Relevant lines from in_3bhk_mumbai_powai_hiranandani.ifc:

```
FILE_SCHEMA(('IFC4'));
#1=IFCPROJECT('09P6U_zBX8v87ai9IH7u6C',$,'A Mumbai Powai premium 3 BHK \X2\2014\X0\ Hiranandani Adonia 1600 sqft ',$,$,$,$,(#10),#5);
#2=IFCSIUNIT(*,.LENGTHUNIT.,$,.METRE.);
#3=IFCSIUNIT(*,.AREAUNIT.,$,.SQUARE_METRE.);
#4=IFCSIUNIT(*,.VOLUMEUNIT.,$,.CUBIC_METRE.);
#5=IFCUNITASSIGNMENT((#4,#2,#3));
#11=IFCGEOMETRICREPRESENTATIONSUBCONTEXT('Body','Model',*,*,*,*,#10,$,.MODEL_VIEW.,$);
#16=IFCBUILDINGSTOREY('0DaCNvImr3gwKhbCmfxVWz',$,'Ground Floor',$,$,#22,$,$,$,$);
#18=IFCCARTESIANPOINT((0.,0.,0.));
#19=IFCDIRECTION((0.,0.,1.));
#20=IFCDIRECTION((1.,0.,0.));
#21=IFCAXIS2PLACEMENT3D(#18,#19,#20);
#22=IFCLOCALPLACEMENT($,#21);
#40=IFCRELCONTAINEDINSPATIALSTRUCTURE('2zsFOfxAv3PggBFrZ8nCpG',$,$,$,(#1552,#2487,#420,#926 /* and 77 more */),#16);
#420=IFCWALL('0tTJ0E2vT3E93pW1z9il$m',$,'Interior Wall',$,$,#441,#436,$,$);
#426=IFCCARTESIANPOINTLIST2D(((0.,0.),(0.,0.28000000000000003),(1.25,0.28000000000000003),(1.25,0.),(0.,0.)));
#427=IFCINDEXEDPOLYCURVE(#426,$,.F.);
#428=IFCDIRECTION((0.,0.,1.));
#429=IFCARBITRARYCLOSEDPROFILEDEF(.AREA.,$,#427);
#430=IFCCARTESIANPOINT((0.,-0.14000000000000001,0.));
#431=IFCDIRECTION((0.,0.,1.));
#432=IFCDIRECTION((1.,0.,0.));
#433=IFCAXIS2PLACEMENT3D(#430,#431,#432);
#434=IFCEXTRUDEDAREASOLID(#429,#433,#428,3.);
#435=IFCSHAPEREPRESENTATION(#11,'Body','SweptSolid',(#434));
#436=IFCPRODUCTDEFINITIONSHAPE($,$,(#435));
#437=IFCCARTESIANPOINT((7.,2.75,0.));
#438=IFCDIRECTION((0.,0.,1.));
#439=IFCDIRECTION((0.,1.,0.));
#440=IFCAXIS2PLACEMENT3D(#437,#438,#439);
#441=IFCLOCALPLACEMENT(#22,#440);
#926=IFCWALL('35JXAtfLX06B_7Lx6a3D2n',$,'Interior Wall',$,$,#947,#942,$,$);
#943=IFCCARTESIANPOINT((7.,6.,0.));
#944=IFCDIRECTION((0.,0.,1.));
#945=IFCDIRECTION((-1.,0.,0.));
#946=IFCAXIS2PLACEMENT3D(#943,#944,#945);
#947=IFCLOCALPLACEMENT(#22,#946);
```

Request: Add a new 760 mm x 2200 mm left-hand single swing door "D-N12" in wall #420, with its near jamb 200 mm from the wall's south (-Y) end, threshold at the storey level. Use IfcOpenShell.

```python
import numpy as np
import ifcopenshell
import ifcopenshell.api.feature
import ifcopenshell.api.geometry
import ifcopenshell.api.root
import ifcopenshell.api.spatial
import ifcopenshell.geom
import ifcopenshell.util.element
import ifcopenshell.util.placement
import ifcopenshell.util.representation
import ifcopenshell.util.shape
import ifcopenshell.util.unit

model = ifcopenshell.open("in_3bhk_mumbai_powai_hiranandani.ifc")
unit_scale = ifcopenshell.util.unit.calculate_unit_scale(model)
settings = ifcopenshell.geom.settings()


def volume(element):
    """Net volume in cubic metres, openings subtracted."""
    shape = ifcopenshell.geom.create_shape(settings, element)
    return ifcopenshell.util.shape.get_volume(shape.geometry)


wall = model.by_id(420)
storey = ifcopenshell.util.element.get_container(wall, ifc_class="IfcBuildingStorey")
context = ifcopenshell.util.representation.get_context(model, "Model", "Body", "MODEL_VIEW")
before = volume(wall)

width, height, from_end, sill = 0.76, 2.2, 0.2, 0.0  # metres

# The wall runs along its own X axis, and the end named is its -X end.
wall_shape = ifcopenshell.geom.create_shape(settings, wall)
x, y, z = ifcopenshell.util.shape.get_vertices(wall_shape.geometry).T
start = x.min() + from_end
face, thickness = float(y.min()), float(y.max() - y.min())
wall_matrix = ifcopenshell.util.placement.get_local_placement(wall.ObjectPlacement)
level = ifcopenshell.util.placement.get_local_placement(storey.ObjectPlacement)[2, 3]


def in_wall(x, y):
    """Placement at x, y metres in the wall's axes, at sill height."""
    matrix = wall_matrix.copy()
    matrix[:, 3] = wall_matrix @ np.array([x / unit_scale, y / unit_scale, 0.0, 1.0])
    matrix[2, 3] = level + sill / unit_scale
    return matrix


# Opening: a box that overshoots both wall faces by 50 mm.
opening = ifcopenshell.api.root.create_entity(model, ifc_class="IfcOpeningElement", predefined_type="OPENING")
box = ifcopenshell.api.geometry.add_wall_representation(
    model, context=context, length=width, height=height, thickness=thickness + 0.1
)
ifcopenshell.api.geometry.assign_representation(model, product=opening, representation=box)
ifcopenshell.api.geometry.edit_object_placement(model, product=opening, matrix=in_wall(start, face - 0.05), is_si=False)
ifcopenshell.api.feature.add_feature(model, feature=opening, element=wall)

door = ifcopenshell.api.root.create_entity(model, ifc_class="IfcDoor", name="D-N12", predefined_type="DOOR")
door.OverallWidth, door.OverallHeight = width / unit_scale, height / unit_scale
door.OperationType = "SINGLE_SWING_LEFT"
body = ifcopenshell.api.geometry.add_door_representation(
    model,
    context=context,
    overall_width=door.OverallWidth,
    overall_height=door.OverallHeight,
    operation_type="SINGLE_SWING_LEFT",
    lining_properties={"LiningDepth": thickness / unit_scale, "ThresholdDepth": thickness / unit_scale},
)
ifcopenshell.api.geometry.assign_representation(model, product=door, representation=body)
ifcopenshell.api.spatial.assign_container(model, products=[door], relating_structure=storey)
ifcopenshell.api.feature.add_filling(model, opening=opening, element=door)

# The lining spans the wall, so the door starts at the wall face.
ifcopenshell.api.geometry.edit_object_placement(model, product=door, matrix=in_wall(start, face), is_si=False)

after = volume(wall)

print(f"wall volume {before:.3f} -> {after:.3f} m3")

model.write("in_3bhk_mumbai_powai_hiranandani_updated.ifc")
```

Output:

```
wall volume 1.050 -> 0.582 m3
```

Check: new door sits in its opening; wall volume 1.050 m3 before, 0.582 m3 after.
